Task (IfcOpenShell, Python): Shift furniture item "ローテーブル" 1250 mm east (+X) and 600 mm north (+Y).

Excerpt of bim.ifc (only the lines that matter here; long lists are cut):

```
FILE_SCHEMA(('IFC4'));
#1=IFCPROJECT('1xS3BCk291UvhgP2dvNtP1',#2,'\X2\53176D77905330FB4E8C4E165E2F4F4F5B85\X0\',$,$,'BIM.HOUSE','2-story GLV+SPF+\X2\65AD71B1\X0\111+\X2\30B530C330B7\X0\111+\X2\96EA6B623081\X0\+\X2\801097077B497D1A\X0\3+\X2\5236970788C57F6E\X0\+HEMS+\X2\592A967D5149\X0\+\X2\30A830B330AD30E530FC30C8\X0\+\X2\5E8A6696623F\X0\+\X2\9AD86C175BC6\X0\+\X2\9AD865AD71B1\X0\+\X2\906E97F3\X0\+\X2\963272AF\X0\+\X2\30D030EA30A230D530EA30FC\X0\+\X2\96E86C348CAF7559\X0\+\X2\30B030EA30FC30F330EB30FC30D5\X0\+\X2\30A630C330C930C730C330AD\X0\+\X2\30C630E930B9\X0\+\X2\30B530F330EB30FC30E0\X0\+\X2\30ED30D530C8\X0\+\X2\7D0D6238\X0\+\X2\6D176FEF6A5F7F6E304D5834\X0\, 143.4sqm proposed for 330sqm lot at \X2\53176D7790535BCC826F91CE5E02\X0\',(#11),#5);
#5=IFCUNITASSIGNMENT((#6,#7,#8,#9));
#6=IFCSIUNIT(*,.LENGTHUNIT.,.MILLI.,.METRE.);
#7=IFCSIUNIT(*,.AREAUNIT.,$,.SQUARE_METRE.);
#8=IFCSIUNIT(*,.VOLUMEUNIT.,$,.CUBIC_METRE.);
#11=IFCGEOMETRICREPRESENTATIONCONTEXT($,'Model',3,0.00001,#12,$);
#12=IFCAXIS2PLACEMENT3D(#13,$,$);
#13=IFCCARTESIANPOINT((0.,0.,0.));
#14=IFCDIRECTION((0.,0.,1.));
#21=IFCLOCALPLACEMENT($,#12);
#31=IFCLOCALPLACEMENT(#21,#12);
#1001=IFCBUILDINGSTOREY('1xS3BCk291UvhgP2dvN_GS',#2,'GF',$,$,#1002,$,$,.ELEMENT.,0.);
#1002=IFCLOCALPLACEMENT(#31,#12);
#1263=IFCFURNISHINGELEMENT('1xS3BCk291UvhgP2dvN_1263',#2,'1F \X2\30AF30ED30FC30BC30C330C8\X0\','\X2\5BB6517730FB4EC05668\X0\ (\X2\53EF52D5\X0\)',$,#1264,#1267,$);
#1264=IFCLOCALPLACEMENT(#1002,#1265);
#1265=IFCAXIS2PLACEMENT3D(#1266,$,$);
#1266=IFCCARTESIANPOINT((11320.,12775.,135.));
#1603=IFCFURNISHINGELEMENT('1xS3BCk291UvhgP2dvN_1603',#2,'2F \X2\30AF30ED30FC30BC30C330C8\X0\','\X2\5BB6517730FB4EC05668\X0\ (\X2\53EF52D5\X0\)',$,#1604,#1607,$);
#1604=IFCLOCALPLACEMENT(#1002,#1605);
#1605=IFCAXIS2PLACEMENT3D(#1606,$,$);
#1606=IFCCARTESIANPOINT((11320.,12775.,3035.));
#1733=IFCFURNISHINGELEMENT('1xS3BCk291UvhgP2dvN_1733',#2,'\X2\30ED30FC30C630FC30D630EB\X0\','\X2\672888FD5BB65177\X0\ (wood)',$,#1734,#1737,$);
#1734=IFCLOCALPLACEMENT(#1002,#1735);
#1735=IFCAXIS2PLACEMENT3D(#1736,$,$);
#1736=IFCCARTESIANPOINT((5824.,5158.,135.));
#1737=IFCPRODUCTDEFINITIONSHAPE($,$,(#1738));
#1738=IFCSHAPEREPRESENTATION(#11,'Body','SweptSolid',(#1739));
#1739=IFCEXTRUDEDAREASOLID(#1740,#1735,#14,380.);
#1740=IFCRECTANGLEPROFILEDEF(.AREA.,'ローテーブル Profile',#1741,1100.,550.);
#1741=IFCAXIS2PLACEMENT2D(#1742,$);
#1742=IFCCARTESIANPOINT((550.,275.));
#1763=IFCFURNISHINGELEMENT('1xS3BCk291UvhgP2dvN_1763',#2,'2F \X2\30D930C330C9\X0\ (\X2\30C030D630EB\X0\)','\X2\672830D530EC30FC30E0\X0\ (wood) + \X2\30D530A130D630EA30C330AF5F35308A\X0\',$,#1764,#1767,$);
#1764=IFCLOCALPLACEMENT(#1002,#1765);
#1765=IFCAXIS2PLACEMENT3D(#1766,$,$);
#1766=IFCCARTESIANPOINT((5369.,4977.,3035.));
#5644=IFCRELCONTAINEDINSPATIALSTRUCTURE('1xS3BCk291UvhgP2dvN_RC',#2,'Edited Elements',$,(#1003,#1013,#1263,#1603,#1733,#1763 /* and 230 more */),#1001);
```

```python
import ifcopenshell
import ifcopenshell.api.geometry
import ifcopenshell.util.placement

model = ifcopenshell.open("bim.ifc")

item = model.by_guid("1xS3BCk291UvhgP2dvN_1733")
matrix = ifcopenshell.util.placement.get_local_placement(item.ObjectPlacement)
matrix[0, 3] += 1250.0
matrix[1, 3] += 600.0
ifcopenshell.api.geometry.edit_object_placement(model, product=item, matrix=matrix, is_si=False)

print(ifcopenshell.util.placement.get_local_placement(item.ObjectPlacement).round(3) + 0.0)

model.write("bim_edited.ifc")
```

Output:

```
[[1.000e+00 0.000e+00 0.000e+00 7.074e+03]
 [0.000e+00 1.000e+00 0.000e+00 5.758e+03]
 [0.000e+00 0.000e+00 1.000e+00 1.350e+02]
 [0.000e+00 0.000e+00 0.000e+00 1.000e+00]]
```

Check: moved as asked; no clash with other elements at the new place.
